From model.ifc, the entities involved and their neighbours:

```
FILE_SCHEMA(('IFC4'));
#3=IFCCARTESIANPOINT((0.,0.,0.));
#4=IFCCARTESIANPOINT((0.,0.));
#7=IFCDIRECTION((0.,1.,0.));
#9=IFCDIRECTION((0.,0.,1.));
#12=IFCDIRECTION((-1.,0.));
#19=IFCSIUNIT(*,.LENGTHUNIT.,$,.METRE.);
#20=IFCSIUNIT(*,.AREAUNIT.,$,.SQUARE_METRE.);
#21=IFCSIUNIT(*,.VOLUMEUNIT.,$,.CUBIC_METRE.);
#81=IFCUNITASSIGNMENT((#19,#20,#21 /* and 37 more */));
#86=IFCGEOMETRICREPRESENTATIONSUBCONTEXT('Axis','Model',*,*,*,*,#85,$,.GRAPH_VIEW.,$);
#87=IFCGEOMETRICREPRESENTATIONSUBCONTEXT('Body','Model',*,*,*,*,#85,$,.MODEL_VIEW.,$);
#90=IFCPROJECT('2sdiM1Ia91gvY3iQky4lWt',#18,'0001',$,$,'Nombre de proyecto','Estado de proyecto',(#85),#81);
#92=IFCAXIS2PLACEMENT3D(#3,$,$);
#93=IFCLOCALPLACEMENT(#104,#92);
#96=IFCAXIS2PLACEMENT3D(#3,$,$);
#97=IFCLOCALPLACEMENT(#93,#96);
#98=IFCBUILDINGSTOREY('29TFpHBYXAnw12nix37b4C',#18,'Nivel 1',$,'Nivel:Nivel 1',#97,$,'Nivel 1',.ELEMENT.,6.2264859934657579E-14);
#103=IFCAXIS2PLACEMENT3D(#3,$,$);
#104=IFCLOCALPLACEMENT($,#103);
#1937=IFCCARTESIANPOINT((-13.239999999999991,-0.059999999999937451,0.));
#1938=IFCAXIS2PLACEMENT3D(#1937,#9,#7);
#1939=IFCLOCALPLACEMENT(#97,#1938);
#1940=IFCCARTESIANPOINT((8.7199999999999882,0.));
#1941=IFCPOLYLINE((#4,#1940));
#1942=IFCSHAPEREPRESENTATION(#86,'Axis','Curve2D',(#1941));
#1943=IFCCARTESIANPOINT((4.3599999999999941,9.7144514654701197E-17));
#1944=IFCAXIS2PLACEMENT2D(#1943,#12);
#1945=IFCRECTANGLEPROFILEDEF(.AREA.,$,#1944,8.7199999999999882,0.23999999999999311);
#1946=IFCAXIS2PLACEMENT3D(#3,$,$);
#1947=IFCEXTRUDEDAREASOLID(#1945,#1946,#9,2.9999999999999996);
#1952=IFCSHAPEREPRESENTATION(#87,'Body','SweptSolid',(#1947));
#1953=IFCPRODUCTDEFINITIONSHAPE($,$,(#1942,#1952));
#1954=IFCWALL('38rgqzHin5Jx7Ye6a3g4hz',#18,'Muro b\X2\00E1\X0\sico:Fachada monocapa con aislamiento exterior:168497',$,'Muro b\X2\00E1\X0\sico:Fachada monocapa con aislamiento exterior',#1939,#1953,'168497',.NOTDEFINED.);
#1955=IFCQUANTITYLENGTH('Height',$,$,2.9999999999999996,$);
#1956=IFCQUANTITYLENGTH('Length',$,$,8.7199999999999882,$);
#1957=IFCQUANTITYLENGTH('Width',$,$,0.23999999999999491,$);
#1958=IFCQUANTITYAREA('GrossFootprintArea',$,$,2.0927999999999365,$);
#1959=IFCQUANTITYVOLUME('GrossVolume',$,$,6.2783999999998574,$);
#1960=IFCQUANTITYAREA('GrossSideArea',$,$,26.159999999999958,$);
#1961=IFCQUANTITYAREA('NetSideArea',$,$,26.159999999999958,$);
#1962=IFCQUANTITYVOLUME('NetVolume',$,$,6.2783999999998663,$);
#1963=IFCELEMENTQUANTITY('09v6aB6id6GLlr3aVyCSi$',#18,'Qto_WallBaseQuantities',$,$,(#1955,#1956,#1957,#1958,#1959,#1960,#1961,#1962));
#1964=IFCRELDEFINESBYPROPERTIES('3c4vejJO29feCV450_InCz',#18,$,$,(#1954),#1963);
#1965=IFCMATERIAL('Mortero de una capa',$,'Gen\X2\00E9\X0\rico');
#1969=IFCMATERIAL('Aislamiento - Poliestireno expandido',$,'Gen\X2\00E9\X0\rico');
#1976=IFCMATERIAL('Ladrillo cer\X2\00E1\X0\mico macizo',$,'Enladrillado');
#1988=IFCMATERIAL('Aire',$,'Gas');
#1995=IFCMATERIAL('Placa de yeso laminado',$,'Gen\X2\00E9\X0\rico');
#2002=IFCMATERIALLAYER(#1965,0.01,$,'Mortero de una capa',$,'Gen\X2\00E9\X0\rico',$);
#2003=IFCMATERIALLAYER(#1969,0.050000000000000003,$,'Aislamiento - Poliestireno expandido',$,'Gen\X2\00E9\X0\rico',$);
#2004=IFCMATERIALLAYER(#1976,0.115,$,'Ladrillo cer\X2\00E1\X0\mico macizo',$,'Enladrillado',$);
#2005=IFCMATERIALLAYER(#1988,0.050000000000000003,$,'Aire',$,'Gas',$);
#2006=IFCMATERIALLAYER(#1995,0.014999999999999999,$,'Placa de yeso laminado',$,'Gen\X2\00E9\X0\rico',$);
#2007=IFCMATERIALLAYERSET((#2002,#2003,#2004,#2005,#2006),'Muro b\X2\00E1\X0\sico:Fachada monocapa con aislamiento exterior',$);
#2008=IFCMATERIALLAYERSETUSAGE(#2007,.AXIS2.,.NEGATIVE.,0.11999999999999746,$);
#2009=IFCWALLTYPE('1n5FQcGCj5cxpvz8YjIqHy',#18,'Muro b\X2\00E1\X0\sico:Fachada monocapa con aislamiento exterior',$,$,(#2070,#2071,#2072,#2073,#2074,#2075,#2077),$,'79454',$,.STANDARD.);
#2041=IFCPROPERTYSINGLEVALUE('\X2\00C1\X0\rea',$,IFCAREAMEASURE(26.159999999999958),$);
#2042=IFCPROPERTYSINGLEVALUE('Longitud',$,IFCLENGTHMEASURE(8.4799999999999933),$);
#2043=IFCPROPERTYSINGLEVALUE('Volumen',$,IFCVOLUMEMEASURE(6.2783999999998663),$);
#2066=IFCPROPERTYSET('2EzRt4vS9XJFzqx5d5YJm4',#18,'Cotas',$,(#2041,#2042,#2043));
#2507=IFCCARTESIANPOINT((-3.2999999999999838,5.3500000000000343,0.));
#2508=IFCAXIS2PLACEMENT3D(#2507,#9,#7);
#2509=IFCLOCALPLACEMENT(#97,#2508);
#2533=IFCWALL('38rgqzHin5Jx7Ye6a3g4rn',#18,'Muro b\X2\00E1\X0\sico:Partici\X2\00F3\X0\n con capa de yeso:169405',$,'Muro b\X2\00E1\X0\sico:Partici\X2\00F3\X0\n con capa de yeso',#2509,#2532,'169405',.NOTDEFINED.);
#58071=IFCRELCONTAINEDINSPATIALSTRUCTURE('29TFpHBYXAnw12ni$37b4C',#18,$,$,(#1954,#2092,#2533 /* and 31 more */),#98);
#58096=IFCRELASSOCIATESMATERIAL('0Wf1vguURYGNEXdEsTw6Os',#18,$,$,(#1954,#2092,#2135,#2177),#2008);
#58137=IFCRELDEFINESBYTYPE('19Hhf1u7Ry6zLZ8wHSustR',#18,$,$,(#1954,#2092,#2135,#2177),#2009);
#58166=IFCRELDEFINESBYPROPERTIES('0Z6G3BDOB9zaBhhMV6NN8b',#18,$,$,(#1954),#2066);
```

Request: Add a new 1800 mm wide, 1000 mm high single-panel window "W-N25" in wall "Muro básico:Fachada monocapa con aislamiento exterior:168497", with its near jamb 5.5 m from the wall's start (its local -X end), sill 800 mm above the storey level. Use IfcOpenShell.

```python
import numpy as np
import ifcopenshell
import ifcopenshell.api.feature
import ifcopenshell.api.geometry
import ifcopenshell.api.pset
import ifcopenshell.api.root
import ifcopenshell.api.spatial
import ifcopenshell.geom
import ifcopenshell.util.element
import ifcopenshell.util.placement
import ifcopenshell.util.representation
import ifcopenshell.util.shape
import ifcopenshell.util.unit

model = ifcopenshell.open("model.ifc")
unit_scale = ifcopenshell.util.unit.calculate_unit_scale(model)
area_scale = ifcopenshell.util.unit.calculate_unit_scale(model, "AREAUNIT")
volume_scale = ifcopenshell.util.unit.calculate_unit_scale(model, "VOLUMEUNIT")
settings = ifcopenshell.geom.settings()


def volume(element):
    """Net volume in cubic metres, openings subtracted."""
    shape = ifcopenshell.geom.create_shape(settings, element)
    return ifcopenshell.util.shape.get_volume(shape.geometry)


wall = model.by_id(1954)
storey = ifcopenshell.util.element.get_container(wall, ifc_class="IfcBuildingStorey")
context = ifcopenshell.util.representation.get_context(model, "Model", "Body", "MODEL_VIEW")
before = volume(wall)

width, height, from_end, sill = 1.8, 1, 5.5, 0.8  # metres

# The wall runs along its own X axis, and the end named is its -X end.
wall_shape = ifcopenshell.geom.create_shape(settings, wall)
x, y, z = ifcopenshell.util.shape.get_vertices(wall_shape.geometry).T
start = x.min() + from_end
face, thickness = float(y.min()), float(y.max() - y.min())
wall_matrix = ifcopenshell.util.placement.get_local_placement(wall.ObjectPlacement)
level = ifcopenshell.util.placement.get_local_placement(storey.ObjectPlacement)[2, 3]


def in_wall(x, y):
    """Placement at x, y metres in the wall's axes, at sill height."""
    matrix = wall_matrix.copy()
    matrix[:, 3] = wall_matrix @ np.array([x / unit_scale, y / unit_scale, 0.0, 1.0])
    matrix[2, 3] = level + sill / unit_scale
    return matrix


# Opening: a box that overshoots both wall faces by 50 mm.
opening = ifcopenshell.api.root.create_entity(model, ifc_class="IfcOpeningElement", predefined_type="OPENING")
box = ifcopenshell.api.geometry.add_wall_representation(
    model, context=context, length=width, height=height, thickness=thickness + 0.1
)
ifcopenshell.api.geometry.assign_representation(model, product=opening, representation=box)
ifcopenshell.api.geometry.edit_object_placement(model, product=opening, matrix=in_wall(start, face - 0.05), is_si=False)
ifcopenshell.api.feature.add_feature(model, feature=opening, element=wall)

window = ifcopenshell.api.root.create_entity(model, ifc_class="IfcWindow", name="W-N25", predefined_type="WINDOW")
window.OverallWidth, window.OverallHeight = width / unit_scale, height / unit_scale
window.PartitioningType = "SINGLE_PANEL"
body = ifcopenshell.api.geometry.add_window_representation(
    model,
    context=context,
    overall_width=window.OverallWidth,
    overall_height=window.OverallHeight,
    partition_type="SINGLE_PANEL",
)
ifcopenshell.api.geometry.assign_representation(model, product=window, representation=body)
ifcopenshell.api.spatial.assign_container(model, products=[window], relating_structure=storey)
ifcopenshell.api.feature.add_filling(model, opening=opening, element=window)

# Centre the window in the wall's thickness.
ifcopenshell.api.geometry.edit_object_placement(model, product=window, matrix=in_wall(start, face), is_si=False)
window_shape = ifcopenshell.geom.create_shape(settings, window)
depth = ifcopenshell.util.shape.get_vertices(window_shape.geometry)[:, 1]
offset = face + thickness / 2 - (depth.min() + depth.max()) / 2
ifcopenshell.api.geometry.edit_object_placement(model, product=window, matrix=in_wall(start, offset), is_si=False)

after = volume(wall)

# Update the wall's stored quantities.
qto = model.by_id(ifcopenshell.util.element.get_pset(wall, "Qto_WallBaseQuantities", should_inherit=False)["id"])
ifcopenshell.api.pset.edit_qto(model, qto=qto, properties={
    "NetSideArea": after / thickness / area_scale,
    "NetVolume": after / volume_scale,
})
pset = model.by_id(ifcopenshell.util.element.get_pset(wall, "Cotas", should_inherit=False)["id"])
ifcopenshell.api.pset.edit_pset(model, pset=pset, properties={
    "Área": model.create_entity("IfcAreaMeasure", after / thickness / area_scale),
    "Volumen": model.create_entity("IfcVolumeMeasure", after / volume_scale),
})

print(f"wall volume {before:.3f} -> {after:.3f} m3")

model.write("model_v2.ifc")
```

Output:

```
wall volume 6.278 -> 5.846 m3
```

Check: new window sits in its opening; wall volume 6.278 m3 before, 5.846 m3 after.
